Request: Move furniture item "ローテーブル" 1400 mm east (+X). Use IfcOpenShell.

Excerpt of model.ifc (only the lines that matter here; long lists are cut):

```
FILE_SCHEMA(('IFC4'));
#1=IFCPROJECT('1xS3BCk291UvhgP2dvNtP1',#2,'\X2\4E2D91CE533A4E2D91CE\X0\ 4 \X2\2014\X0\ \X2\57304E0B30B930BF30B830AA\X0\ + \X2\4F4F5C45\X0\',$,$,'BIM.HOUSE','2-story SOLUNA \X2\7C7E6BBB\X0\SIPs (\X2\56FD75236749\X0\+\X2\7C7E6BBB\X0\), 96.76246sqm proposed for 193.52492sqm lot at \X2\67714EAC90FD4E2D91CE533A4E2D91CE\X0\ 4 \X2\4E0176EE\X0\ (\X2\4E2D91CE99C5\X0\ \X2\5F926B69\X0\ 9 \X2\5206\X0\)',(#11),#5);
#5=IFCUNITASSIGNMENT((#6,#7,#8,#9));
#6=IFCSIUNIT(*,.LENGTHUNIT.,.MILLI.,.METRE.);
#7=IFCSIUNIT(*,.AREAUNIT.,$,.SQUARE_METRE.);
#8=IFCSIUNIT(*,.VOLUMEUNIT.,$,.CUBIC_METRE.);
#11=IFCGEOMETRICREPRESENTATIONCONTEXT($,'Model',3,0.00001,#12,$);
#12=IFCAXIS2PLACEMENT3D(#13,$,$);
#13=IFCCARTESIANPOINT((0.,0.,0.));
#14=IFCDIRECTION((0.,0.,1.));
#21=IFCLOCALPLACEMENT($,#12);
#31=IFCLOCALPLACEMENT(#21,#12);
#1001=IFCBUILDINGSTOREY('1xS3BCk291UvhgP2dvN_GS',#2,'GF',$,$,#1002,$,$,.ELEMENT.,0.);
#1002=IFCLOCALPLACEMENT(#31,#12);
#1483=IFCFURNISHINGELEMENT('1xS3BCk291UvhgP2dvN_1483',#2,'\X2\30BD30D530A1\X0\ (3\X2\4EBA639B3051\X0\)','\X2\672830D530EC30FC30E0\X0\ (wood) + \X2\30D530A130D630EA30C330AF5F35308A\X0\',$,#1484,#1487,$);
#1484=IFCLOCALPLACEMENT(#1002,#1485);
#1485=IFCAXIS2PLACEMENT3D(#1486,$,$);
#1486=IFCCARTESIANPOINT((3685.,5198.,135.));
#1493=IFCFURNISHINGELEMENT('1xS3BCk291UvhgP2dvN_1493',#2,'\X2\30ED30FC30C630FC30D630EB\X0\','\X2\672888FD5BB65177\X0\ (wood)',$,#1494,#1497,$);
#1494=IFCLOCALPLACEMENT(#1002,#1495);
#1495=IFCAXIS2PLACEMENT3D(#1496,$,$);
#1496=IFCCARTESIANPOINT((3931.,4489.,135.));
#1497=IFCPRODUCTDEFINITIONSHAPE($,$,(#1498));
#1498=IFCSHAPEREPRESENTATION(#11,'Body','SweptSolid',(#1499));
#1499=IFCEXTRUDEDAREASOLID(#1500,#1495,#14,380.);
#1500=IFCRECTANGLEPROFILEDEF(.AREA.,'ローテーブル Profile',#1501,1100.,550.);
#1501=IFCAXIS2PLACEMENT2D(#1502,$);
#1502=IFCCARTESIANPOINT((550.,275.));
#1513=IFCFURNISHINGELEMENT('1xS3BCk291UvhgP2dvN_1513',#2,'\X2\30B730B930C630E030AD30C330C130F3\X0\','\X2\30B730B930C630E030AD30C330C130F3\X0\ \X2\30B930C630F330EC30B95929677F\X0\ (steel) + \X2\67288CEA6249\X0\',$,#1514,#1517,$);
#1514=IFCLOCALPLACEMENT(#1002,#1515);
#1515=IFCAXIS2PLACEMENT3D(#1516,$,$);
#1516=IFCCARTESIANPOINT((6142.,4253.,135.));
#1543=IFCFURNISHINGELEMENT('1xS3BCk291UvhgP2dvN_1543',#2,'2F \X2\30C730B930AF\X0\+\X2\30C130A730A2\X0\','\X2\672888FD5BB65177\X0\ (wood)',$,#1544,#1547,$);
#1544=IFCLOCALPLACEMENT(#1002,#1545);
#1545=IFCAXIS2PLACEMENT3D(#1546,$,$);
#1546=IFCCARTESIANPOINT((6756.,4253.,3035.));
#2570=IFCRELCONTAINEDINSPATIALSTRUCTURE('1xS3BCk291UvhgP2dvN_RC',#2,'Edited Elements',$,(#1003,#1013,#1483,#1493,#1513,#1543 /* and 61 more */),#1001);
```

```python
import ifcopenshell
import ifcopenshell.api.geometry
import ifcopenshell.util.placement
import ifcopenshell.util.unit

model = ifcopenshell.open("model.ifc")
unit_scale = ifcopenshell.util.unit.calculate_unit_scale(model)

item = model.by_guid("1xS3BCk291UvhgP2dvN_1493")
matrix = ifcopenshell.util.placement.get_local_placement(item.ObjectPlacement)
matrix[0, 3] += 1.4 / unit_scale
ifcopenshell.api.geometry.edit_object_placement(model, product=item, matrix=matrix, is_si=False)

print(ifcopenshell.util.placement.get_local_placement(item.ObjectPlacement).round(3) + 0.0)

model.write("model_updated.ifc")
```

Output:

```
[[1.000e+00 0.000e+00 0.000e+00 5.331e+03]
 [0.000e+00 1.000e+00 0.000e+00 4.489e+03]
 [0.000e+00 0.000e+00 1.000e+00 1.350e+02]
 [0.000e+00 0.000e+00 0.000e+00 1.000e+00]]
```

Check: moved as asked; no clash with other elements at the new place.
